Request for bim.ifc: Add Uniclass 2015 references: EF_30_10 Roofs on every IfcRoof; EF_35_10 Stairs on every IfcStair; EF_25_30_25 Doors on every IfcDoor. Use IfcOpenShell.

First a look at what the model holds.

```python
import ifcopenshell

model = ifcopenshell.open("bim.ifc")
print(model.schema)
print("classifications:", [c.Name for c in model.by_type("IfcClassification")])
for ifc_class in ("IfcDoor", "IfcRoof", "IfcStair", "IfcWall", "IfcWindow"):
    print(ifc_class, len(model.by_type(ifc_class)))
```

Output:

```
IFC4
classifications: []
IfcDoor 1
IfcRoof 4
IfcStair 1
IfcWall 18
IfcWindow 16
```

```python
import ifcopenshell
import ifcopenshell.api.classification

model = ifcopenshell.open("bim.ifc")

system = ifcopenshell.api.classification.add_classification(model, classification="Uniclass 2015")

codes = {
    "IfcRoof": ("EF_30_10", "Roofs"),
    "IfcStair": ("EF_35_10", "Stairs"),
    "IfcDoor": ("EF_25_30_25", "Doors"),
}
for ifc_class, (code, name) in codes.items():
    products = model.by_type(ifc_class)
    ifcopenshell.api.classification.add_reference(
        model, products=products, classification=system, identification=code, name=name
    )
    print(code, len(products))

model.write("bim_v2.ifc")
```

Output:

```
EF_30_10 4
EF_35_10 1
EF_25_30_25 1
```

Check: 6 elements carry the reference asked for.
